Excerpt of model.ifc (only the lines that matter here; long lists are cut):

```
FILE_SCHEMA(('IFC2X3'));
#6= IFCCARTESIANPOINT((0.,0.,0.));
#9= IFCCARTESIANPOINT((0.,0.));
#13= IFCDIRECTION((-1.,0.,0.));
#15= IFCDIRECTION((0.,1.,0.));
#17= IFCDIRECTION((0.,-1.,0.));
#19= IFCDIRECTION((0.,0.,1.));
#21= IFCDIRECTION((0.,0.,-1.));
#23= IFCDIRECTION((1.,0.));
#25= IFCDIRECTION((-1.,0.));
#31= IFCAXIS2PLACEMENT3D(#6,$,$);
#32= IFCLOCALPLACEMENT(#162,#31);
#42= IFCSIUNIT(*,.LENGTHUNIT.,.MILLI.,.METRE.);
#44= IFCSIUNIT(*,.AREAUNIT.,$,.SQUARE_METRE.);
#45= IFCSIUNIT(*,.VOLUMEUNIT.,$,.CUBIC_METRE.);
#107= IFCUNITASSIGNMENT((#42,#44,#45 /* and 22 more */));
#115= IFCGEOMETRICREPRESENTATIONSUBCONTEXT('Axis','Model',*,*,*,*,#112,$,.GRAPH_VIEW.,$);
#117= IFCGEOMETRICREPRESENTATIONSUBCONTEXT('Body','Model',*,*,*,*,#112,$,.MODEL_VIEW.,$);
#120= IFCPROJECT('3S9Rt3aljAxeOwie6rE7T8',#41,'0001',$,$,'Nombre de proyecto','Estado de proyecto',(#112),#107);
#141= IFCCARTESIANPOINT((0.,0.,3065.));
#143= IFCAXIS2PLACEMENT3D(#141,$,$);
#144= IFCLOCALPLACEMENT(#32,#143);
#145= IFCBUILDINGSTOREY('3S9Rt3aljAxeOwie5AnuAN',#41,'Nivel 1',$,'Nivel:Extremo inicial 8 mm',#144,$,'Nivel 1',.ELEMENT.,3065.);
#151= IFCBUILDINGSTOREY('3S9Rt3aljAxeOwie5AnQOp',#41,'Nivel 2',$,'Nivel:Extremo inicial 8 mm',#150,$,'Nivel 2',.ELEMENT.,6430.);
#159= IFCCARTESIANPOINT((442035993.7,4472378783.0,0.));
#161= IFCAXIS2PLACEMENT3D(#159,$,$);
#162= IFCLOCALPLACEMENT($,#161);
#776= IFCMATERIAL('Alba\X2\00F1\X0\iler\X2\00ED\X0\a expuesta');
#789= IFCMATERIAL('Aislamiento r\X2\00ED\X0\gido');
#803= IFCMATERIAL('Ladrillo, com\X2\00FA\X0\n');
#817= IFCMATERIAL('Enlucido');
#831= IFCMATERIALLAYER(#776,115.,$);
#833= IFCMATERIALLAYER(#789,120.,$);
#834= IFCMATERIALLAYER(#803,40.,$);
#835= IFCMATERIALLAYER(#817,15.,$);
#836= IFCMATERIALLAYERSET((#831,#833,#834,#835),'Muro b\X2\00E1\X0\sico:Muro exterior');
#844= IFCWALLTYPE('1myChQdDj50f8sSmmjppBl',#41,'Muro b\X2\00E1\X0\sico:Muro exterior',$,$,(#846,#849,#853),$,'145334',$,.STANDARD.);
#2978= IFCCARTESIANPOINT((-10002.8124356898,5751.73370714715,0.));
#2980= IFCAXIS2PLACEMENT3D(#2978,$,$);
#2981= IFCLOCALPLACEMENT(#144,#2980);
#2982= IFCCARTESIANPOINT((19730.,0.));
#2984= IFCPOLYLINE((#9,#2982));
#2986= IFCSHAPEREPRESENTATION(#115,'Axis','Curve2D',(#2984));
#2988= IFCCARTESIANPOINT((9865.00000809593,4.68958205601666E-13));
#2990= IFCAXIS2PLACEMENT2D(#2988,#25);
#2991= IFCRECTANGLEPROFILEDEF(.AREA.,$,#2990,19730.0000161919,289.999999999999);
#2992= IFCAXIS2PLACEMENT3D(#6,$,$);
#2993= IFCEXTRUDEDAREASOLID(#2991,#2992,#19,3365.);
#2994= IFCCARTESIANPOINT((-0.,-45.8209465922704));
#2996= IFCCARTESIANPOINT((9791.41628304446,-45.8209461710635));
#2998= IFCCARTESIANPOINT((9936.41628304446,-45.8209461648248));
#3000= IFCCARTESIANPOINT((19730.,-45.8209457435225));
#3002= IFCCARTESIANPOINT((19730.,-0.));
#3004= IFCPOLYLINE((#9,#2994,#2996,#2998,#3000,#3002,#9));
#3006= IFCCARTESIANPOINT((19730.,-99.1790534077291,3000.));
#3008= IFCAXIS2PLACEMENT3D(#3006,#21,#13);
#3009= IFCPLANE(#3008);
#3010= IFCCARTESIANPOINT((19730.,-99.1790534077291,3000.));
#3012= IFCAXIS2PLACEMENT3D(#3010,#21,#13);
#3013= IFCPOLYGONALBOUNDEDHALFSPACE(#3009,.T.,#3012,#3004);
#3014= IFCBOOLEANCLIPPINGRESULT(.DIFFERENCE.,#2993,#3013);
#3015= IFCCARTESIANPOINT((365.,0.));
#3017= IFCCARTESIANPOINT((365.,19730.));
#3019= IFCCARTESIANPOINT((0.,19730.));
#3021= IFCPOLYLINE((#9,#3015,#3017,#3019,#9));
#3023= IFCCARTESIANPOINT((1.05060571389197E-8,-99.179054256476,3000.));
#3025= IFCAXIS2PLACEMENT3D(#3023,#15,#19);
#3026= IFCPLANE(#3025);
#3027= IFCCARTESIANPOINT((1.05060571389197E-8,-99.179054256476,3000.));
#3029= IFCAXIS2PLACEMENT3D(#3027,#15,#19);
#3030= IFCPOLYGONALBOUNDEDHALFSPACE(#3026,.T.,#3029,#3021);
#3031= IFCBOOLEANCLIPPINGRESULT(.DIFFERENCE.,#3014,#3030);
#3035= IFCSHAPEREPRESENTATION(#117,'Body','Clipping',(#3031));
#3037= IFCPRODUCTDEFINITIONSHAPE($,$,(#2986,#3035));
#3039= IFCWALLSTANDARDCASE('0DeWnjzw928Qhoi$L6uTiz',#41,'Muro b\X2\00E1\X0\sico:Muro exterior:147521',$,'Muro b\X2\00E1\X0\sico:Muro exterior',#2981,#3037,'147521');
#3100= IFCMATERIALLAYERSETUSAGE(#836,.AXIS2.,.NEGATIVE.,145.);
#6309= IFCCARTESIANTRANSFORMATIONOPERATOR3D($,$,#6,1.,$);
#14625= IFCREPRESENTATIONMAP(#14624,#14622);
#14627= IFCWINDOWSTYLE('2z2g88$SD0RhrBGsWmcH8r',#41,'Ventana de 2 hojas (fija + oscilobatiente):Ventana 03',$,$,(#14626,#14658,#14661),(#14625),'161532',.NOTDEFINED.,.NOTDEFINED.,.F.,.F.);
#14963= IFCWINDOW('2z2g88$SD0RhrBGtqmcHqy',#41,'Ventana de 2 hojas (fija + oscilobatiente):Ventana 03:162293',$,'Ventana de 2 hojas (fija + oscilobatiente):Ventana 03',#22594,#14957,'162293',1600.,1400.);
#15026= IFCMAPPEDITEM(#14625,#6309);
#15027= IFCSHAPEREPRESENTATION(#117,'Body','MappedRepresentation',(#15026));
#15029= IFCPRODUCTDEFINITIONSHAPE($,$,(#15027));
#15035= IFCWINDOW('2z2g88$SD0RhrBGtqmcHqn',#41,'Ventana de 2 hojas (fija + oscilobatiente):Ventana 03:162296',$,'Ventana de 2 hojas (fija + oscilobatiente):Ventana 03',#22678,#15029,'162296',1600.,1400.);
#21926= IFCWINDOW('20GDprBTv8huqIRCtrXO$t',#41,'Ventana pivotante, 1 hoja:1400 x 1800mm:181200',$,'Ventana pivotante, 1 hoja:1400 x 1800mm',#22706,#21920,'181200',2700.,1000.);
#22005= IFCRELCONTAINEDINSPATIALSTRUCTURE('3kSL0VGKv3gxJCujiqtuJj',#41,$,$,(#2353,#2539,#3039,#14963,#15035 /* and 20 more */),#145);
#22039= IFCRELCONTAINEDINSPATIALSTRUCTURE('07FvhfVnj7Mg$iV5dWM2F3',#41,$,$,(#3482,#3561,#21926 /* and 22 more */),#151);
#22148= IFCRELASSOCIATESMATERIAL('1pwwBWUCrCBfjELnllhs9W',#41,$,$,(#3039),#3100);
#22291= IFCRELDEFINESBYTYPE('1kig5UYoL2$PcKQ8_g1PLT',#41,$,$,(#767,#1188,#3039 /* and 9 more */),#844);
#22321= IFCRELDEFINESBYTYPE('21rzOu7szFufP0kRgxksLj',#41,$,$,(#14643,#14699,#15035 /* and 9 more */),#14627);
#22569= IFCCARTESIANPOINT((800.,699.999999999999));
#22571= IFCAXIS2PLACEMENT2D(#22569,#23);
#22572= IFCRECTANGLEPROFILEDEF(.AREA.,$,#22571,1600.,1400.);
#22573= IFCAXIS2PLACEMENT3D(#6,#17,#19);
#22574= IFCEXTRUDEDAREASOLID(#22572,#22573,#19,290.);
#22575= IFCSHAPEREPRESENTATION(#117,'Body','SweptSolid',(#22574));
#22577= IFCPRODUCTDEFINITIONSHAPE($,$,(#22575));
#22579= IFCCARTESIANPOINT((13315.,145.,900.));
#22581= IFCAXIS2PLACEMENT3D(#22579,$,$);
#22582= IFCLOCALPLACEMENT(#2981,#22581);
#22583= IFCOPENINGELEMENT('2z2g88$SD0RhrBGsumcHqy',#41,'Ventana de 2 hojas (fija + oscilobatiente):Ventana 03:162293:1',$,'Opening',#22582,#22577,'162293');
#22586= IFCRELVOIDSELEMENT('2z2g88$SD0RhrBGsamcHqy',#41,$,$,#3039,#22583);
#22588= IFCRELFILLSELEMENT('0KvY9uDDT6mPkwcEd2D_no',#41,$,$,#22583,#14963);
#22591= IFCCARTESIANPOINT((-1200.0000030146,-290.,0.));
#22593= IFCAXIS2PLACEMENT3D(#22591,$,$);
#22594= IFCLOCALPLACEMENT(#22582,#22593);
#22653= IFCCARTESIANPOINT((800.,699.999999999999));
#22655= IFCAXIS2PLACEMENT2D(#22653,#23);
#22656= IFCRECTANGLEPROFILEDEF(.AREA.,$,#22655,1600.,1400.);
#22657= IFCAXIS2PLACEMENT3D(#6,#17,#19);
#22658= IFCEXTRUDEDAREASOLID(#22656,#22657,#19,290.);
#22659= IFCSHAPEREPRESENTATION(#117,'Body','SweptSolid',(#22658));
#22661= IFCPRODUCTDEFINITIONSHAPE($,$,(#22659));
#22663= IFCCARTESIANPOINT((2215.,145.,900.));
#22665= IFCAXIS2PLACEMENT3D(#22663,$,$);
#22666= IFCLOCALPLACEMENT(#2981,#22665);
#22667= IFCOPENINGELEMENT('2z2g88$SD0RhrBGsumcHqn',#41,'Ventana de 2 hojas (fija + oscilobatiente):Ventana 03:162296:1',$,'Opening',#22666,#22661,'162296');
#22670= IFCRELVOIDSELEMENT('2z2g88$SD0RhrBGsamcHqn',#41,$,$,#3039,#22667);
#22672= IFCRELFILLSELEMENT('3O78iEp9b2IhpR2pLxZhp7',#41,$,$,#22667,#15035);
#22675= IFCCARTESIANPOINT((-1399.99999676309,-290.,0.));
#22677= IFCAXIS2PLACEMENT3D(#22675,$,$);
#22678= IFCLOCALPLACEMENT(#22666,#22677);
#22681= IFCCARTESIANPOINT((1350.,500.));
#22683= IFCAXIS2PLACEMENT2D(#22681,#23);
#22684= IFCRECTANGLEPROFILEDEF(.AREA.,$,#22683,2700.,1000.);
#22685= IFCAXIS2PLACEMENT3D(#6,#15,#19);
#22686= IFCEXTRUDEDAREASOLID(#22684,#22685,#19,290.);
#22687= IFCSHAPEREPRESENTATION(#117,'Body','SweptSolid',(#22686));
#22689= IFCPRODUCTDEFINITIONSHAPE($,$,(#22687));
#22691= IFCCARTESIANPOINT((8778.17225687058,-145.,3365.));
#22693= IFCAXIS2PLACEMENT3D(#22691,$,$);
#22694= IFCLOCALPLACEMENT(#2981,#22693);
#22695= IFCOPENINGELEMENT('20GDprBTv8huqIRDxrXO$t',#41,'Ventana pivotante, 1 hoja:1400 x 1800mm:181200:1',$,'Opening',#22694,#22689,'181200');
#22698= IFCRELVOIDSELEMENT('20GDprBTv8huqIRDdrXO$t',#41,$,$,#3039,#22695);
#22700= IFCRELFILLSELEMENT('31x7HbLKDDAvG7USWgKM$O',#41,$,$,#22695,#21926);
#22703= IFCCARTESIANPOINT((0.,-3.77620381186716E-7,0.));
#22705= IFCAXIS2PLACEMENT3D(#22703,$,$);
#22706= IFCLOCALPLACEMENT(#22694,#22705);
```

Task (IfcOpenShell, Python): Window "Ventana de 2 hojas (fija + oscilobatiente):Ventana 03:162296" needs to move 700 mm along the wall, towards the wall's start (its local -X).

```python
import ifcopenshell
import ifcopenshell.api.geometry
import ifcopenshell.util.placement
import ifcopenshell.util.unit

model = ifcopenshell.open("model.ifc")
unit_scale = ifcopenshell.util.unit.calculate_unit_scale(model)

window = model.by_id(15035)
opening = window.FillsVoids[0].RelatingOpeningElement
wall = opening.VoidsElements[0].RelatingBuildingElement

wall_matrix = ifcopenshell.util.placement.get_local_placement(wall.ObjectPlacement)
shift = wall_matrix[:3, 0] * -0.7 / unit_scale
before = ifcopenshell.util.placement.get_local_placement(window.ObjectPlacement)[:3, 3].copy()

# The window is placed relative to its opening, so it follows when the opening moves.
matrix = ifcopenshell.util.placement.get_local_placement(opening.ObjectPlacement)
matrix[:3, 3] += shift
ifcopenshell.api.geometry.edit_object_placement(
    model, product=opening, matrix=matrix, is_si=False, should_transform_children=True
)

after = ifcopenshell.util.placement.get_local_placement(window.ObjectPlacement)[:3, 3]
print("window moved by", (after - before).round(3) + 0.0)

model.write("model_rev.ifc")
```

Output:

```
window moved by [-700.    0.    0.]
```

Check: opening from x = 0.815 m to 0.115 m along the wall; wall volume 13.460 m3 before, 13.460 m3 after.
